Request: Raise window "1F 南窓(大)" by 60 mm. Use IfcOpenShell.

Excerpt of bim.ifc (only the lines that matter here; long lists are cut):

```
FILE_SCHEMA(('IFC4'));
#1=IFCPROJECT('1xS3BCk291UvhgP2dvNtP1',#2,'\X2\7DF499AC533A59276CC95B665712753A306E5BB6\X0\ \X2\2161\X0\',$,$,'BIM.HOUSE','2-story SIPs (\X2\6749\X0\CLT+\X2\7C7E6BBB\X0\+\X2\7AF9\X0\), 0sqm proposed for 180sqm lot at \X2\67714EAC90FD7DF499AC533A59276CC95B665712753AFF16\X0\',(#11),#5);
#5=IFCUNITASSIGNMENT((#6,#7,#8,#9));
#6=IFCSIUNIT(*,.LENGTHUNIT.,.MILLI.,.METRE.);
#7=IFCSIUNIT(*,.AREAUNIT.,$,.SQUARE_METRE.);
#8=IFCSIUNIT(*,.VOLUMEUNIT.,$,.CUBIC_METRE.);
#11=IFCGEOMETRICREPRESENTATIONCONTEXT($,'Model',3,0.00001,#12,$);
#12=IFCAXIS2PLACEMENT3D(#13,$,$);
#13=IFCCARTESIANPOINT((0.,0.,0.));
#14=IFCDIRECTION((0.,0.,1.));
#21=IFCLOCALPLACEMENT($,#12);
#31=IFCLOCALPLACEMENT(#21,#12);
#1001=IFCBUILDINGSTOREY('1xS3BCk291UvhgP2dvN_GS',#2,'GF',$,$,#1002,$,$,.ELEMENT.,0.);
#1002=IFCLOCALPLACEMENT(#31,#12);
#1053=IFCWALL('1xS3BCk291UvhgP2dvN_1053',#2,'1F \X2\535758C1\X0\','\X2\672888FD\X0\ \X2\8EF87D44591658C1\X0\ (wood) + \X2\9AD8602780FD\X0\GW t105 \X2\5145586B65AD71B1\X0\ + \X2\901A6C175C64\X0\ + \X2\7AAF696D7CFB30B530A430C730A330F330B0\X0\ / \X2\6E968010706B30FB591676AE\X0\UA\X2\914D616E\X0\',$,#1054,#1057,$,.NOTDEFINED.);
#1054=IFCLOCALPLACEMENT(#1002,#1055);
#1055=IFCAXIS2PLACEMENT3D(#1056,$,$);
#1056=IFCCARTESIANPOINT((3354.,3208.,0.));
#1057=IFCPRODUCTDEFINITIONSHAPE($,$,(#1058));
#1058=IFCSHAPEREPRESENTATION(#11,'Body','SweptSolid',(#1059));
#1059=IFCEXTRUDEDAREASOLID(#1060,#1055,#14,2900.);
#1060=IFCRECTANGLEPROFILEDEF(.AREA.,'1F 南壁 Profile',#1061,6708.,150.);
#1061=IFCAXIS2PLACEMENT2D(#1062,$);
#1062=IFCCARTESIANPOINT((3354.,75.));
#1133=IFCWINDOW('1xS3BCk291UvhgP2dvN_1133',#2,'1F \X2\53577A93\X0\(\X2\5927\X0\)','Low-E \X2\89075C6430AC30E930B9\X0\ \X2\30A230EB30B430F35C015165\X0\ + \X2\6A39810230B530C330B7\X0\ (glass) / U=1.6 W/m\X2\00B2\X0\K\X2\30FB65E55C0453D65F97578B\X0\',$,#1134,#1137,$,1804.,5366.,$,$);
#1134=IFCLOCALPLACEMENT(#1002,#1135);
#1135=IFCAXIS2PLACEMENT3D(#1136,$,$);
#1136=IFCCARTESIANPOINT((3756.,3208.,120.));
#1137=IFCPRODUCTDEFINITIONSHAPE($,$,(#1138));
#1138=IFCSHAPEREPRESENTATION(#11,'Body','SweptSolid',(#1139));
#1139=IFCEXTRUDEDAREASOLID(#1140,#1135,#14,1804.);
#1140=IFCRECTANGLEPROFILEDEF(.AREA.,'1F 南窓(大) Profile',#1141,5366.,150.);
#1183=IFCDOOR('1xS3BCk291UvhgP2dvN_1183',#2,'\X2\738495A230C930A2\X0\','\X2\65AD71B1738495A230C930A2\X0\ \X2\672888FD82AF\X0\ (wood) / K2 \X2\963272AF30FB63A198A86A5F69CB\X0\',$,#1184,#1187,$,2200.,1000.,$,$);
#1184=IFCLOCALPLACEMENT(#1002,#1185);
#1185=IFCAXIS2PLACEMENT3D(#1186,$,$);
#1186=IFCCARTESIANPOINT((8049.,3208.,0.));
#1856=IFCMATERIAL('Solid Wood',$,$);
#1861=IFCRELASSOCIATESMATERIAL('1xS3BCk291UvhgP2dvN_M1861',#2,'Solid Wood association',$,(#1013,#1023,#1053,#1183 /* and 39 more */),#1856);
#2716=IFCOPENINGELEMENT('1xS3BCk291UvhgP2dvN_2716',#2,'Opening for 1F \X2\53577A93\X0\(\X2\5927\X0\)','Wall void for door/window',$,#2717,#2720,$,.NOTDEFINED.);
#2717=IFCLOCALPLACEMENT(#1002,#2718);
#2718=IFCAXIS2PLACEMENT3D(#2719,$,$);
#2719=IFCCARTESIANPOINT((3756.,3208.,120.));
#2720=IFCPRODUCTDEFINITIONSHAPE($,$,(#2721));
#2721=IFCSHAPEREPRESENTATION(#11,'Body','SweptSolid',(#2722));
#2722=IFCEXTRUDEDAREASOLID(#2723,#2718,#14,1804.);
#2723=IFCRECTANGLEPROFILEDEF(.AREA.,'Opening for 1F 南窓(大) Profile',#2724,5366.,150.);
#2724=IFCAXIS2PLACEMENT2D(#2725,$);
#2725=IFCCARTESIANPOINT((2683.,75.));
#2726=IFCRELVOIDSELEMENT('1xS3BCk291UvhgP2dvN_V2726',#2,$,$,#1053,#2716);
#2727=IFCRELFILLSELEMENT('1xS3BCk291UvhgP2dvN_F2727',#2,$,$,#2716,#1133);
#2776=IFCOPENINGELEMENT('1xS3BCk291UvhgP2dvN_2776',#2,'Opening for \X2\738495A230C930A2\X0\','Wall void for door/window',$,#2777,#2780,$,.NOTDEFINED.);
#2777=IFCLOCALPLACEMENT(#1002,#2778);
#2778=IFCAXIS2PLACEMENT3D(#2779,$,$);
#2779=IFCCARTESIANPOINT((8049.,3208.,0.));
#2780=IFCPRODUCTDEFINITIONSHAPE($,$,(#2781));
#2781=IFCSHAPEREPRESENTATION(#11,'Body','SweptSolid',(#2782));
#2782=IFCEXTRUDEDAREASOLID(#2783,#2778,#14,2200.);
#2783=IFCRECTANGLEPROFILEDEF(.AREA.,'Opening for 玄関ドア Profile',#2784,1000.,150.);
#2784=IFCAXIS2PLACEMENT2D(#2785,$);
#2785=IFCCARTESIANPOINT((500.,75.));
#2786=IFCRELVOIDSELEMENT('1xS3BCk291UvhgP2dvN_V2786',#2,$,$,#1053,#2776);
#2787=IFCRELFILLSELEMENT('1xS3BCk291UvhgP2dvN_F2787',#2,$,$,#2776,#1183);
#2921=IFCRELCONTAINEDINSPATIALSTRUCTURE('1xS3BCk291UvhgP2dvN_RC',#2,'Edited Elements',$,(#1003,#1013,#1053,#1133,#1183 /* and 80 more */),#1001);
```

```python
import numpy as np
import ifcopenshell
import ifcopenshell.api.geometry
import ifcopenshell.util.placement
import ifcopenshell.util.unit

model = ifcopenshell.open("bim.ifc")
unit_scale = ifcopenshell.util.unit.calculate_unit_scale(model)

window = model.by_guid("1xS3BCk291UvhgP2dvN_1133")
opening = window.FillsVoids[0].RelatingOpeningElement
dz = 0.06 / unit_scale

shift = np.array([0.0, 0.0, dz])
# The window is not placed relative to its opening, so move both.
for product in (opening, window):
    matrix = ifcopenshell.util.placement.get_local_placement(product.ObjectPlacement)
    matrix[:3, 3] += shift
    ifcopenshell.api.geometry.edit_object_placement(model, product=product, matrix=matrix, is_si=False)

print(f"moved by {dz * unit_scale:+.3f} m")

model.write("bim_rev.ifc")
```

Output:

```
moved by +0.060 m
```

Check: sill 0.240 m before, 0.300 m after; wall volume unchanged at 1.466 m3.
